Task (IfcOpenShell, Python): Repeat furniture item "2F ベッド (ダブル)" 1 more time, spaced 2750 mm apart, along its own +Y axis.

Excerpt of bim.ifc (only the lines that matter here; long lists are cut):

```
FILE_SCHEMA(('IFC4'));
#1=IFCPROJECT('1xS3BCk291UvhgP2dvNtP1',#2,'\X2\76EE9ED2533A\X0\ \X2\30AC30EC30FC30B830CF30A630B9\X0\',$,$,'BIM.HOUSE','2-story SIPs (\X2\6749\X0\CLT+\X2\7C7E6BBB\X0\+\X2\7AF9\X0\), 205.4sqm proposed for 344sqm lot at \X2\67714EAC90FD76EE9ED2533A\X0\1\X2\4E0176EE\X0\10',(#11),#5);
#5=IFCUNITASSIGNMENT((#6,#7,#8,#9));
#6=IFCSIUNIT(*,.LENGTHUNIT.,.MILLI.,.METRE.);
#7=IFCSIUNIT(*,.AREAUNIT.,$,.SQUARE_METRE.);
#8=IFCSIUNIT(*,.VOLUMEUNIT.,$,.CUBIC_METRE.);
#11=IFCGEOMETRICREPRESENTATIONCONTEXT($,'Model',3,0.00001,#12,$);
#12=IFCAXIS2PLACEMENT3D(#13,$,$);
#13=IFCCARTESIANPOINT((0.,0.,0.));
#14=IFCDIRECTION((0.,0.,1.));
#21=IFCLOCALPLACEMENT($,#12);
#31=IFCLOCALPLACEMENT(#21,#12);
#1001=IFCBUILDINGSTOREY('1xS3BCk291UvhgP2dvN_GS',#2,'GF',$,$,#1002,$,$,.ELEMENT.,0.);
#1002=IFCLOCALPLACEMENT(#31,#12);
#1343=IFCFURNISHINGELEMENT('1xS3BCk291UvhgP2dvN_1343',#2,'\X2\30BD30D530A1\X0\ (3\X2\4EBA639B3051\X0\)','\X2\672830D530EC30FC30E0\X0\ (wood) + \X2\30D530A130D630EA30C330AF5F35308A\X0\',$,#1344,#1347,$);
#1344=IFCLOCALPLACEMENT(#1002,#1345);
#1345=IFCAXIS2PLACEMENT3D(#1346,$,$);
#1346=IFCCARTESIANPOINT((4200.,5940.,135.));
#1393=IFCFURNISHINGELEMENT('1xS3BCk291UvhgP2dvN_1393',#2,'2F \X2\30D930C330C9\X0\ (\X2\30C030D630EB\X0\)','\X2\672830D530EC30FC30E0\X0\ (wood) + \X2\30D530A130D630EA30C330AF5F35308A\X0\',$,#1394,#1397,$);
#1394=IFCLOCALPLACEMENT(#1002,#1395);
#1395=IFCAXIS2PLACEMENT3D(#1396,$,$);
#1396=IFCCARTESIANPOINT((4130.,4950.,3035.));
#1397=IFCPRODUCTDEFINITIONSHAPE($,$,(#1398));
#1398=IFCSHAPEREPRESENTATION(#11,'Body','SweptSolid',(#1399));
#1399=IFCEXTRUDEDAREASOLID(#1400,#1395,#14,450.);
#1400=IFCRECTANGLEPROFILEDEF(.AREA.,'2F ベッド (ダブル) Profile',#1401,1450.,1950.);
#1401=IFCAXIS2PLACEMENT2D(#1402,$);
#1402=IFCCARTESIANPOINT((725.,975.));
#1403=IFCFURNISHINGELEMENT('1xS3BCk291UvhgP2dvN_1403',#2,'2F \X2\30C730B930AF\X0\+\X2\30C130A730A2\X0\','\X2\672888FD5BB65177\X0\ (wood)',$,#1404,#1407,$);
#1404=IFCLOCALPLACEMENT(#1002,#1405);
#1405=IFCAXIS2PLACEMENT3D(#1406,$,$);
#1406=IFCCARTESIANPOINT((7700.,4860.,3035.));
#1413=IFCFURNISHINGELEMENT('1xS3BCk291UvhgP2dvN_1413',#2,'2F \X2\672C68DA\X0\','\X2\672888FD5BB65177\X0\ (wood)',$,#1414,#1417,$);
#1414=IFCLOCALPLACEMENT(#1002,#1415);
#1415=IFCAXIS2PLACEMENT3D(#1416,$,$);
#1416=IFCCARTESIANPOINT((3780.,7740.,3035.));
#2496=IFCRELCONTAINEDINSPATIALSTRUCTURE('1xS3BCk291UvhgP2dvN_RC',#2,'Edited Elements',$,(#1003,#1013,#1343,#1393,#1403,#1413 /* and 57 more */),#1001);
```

```python
import ifcopenshell
import ifcopenshell.api.geometry
import ifcopenshell.api.root
import ifcopenshell.util.element
import ifcopenshell.util.placement
import ifcopenshell.util.unit

model = ifcopenshell.open("bim.ifc")
unit_scale = ifcopenshell.util.unit.calculate_unit_scale(model)


def reuse_history(source, copy):
    """copy_class also copies each property set's owner history, people and application; keep the originals."""
    for rel in copy.IsDefinedBy:
        if rel.is_a("IfcRelDefinesByProperties") and (history := rel.RelatingPropertyDefinition.OwnerHistory):
            rel.RelatingPropertyDefinition.OwnerHistory = source.OwnerHistory
            ifcopenshell.util.element.remove_deep2(model, history)


source = model.by_id(1393)
base = ifcopenshell.util.placement.get_local_placement(source.ObjectPlacement)
step = base[:3, 1] * 2.75 / unit_scale

for i in range(1, 2):
    copy = ifcopenshell.api.root.copy_class(model, product=source)
    copy.Representation = ifcopenshell.util.element.copy_deep(
        model, source.Representation, exclude=["IfcGeometricRepresentationContext", "IfcRepresentationMap"]
    )
    reuse_history(source, copy)
    matrix = base.copy()
    matrix[:3, 3] += i * step
    print("added at", matrix[:3, 3].round(3) + 0.0)
    ifcopenshell.api.geometry.edit_object_placement(model, product=copy, matrix=matrix, is_si=False)

model.write("bim_updated.ifc")
```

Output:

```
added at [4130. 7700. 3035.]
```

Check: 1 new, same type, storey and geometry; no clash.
